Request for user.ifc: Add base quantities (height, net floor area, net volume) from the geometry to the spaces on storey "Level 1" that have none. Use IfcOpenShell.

First a look at what the model holds.

```python
import ifcopenshell
import ifcopenshell.util.element
import ifcopenshell.util.unit

model = ifcopenshell.open("user.ifc")
print(model.schema)
for unit_type in ("LENGTHUNIT", "AREAUNIT", "VOLUMEUNIT"):
    print(unit_type, ifcopenshell.util.unit.calculate_unit_scale(model, unit_type))
storey = next(s for s in model.by_type("IfcBuildingStorey") if s.Name == "Level 1")
spaces = [e for e in ifcopenshell.util.element.get_decomposition(storey) if e.is_a("IfcSpace")]
for e in sorted(spaces, key=lambda e: e.id()):
    print(e.id(), e.is_a(), e.Name, list(ifcopenshell.util.element.get_psets(e, qtos_only=True)), sep=" | ")
```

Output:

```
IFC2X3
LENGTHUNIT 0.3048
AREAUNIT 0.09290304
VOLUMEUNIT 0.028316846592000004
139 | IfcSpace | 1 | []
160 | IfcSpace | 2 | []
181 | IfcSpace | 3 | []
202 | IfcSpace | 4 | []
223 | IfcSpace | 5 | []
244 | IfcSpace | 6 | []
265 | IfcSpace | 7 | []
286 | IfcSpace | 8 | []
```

```python
import ifcopenshell
import ifcopenshell.api.pset
import ifcopenshell.geom
import ifcopenshell.util.element
import ifcopenshell.util.shape
import ifcopenshell.util.unit

model = ifcopenshell.open("user.ifc")
unit_scale = ifcopenshell.util.unit.calculate_unit_scale(model)
area_scale = ifcopenshell.util.unit.calculate_unit_scale(model, "AREAUNIT")
volume_scale = ifcopenshell.util.unit.calculate_unit_scale(model, "VOLUMEUNIT")
settings = ifcopenshell.geom.settings()

storey = next(s for s in model.by_type("IfcBuildingStorey") if s.Name == "Level 1")
spaces = [e for e in ifcopenshell.util.element.get_decomposition(storey) if e.is_a("IfcSpace")]

for e in sorted(spaces, key=lambda e: e.id()):
    if ifcopenshell.util.element.get_psets(e, qtos_only=True, should_inherit=False):
        continue
    # Geometry comes back in metres, in the element's own axes.
    shape = ifcopenshell.geom.create_shape(settings, e)
    values = {
        "Height": ifcopenshell.util.shape.get_z(shape.geometry) / unit_scale,
        "NetFloorArea": ifcopenshell.util.shape.get_footprint_area(shape.geometry) / area_scale,
        "NetVolume": ifcopenshell.util.shape.get_volume(shape.geometry) / volume_scale,
    }
    qto = ifcopenshell.api.pset.add_qto(model, product=e, name="BaseQuantities")
    ifcopenshell.api.pset.edit_qto(model, qto=qto, properties=values)
    print(e.id(), {k: round(v, 3) for k, v in values.items()})

model.write("user-out.ifc")
```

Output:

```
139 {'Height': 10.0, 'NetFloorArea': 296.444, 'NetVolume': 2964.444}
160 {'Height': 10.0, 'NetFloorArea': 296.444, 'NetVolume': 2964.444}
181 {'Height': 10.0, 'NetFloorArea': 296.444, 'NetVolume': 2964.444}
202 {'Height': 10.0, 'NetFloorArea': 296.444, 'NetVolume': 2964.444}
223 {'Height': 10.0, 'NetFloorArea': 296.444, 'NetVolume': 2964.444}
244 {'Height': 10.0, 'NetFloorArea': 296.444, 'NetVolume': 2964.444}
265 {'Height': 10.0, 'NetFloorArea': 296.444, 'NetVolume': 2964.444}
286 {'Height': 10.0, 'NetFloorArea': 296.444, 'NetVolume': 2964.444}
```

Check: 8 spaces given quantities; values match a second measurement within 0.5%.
